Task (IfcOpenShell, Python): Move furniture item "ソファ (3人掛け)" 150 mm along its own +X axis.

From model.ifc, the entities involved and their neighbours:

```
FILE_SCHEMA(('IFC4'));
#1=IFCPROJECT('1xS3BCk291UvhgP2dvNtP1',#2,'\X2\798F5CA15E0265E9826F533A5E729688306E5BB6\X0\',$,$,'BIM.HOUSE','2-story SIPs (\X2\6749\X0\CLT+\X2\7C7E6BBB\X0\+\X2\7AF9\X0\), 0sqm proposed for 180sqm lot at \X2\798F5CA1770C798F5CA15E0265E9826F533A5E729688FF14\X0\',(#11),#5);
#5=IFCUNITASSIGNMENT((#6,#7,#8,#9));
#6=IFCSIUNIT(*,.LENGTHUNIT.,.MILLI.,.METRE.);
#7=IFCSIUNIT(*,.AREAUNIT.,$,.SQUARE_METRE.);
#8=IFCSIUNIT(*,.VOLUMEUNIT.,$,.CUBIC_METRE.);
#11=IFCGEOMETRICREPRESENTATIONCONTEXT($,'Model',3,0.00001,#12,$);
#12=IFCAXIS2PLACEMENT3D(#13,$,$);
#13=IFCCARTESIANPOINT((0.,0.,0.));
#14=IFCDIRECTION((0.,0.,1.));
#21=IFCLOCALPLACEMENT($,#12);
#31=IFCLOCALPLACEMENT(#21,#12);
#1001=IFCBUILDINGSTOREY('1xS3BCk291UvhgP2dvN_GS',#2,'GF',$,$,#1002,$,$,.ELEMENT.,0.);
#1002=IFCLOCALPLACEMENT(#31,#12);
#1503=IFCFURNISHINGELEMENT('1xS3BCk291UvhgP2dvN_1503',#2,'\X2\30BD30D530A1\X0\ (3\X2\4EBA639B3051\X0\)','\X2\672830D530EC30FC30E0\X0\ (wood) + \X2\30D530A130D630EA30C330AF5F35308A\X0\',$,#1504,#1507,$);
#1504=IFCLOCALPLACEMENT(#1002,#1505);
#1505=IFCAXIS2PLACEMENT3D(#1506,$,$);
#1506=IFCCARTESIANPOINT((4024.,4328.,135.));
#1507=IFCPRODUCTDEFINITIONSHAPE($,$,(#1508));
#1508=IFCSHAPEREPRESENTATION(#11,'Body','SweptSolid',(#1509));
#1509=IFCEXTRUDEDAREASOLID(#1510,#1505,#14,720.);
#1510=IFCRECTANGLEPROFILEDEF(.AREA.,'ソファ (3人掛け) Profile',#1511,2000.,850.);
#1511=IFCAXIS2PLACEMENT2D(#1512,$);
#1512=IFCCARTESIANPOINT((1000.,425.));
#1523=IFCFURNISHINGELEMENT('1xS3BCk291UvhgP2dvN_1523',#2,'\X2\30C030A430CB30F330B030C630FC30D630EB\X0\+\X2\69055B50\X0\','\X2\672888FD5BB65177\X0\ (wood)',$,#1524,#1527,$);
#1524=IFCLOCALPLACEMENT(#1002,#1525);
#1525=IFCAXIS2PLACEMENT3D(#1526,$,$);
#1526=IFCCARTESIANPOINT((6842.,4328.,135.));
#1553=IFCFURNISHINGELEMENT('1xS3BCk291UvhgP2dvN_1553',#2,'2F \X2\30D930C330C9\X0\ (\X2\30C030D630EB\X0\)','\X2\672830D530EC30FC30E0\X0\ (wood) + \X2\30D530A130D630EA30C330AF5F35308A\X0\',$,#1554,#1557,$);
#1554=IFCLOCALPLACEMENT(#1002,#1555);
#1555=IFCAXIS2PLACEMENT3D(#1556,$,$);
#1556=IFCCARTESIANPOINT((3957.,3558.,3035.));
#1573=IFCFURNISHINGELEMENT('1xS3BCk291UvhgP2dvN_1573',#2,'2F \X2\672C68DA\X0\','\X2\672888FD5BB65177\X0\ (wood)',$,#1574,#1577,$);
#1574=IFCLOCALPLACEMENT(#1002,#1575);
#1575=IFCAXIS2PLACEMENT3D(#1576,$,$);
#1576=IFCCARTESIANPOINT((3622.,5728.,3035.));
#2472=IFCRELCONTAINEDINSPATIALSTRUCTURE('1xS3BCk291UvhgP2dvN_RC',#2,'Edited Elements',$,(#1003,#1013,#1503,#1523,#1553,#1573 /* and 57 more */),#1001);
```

```python
import ifcopenshell
import ifcopenshell.api.geometry
import ifcopenshell.util.placement

model = ifcopenshell.open("model.ifc")

item = model.by_id(1503)
matrix = ifcopenshell.util.placement.get_local_placement(item.ObjectPlacement)
matrix[:3, 3] += matrix[:3, 0] * 150.0
ifcopenshell.api.geometry.edit_object_placement(model, product=item, matrix=matrix, is_si=False)

print(ifcopenshell.util.placement.get_local_placement(item.ObjectPlacement).round(3) + 0.0)

model.write("model_edited.ifc")
```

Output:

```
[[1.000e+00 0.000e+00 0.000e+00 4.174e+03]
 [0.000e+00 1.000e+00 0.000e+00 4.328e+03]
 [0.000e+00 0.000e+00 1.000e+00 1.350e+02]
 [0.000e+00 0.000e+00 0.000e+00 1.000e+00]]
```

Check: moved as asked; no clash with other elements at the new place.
